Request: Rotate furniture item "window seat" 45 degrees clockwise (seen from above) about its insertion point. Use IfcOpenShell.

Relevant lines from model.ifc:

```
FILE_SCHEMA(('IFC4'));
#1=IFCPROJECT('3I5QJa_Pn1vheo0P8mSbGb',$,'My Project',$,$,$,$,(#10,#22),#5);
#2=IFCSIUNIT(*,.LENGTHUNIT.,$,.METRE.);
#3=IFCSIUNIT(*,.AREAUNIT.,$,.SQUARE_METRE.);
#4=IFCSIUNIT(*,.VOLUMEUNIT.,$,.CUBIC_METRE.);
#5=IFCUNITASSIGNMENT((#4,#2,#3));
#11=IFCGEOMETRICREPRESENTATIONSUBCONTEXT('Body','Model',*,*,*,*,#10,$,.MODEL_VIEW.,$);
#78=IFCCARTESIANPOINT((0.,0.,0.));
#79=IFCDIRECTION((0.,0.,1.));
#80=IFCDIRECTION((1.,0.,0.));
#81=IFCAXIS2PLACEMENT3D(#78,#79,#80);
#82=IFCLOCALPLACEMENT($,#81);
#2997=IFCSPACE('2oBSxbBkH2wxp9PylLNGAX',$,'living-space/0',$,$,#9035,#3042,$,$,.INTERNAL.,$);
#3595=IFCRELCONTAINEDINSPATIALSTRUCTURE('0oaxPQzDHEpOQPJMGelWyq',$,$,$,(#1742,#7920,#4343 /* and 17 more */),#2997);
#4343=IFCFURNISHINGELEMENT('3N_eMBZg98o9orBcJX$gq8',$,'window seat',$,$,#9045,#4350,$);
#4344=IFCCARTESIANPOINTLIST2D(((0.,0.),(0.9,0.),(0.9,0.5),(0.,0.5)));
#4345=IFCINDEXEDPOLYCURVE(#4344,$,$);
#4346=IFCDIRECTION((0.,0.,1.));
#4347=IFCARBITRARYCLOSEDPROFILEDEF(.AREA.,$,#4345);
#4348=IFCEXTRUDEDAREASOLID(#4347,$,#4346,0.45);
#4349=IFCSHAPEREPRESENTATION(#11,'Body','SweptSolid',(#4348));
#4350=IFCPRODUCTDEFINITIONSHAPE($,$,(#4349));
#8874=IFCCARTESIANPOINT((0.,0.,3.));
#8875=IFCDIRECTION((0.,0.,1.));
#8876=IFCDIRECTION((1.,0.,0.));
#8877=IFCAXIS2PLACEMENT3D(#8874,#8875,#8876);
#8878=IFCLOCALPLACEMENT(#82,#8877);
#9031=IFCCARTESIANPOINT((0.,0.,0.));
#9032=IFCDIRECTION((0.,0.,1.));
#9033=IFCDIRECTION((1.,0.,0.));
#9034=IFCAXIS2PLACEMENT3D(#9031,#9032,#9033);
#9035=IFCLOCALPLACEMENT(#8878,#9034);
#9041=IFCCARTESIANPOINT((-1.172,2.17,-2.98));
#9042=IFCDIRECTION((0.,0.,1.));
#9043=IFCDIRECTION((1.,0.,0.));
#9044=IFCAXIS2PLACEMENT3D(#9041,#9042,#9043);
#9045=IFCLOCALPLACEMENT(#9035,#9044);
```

```python
import ifcopenshell
import ifcopenshell.api.geometry
import ifcopenshell.util.placement

model = ifcopenshell.open("model.ifc")

item = model.by_id(4343)
matrix = ifcopenshell.util.placement.get_local_placement(item.ObjectPlacement)
matrix = matrix @ ifcopenshell.util.placement.rotation(-45, "Z")
ifcopenshell.api.geometry.edit_object_placement(model, product=item, matrix=matrix, is_si=False)

print(ifcopenshell.util.placement.get_local_placement(item.ObjectPlacement).round(3) + 0.0)

model.write("model_v2.ifc")
```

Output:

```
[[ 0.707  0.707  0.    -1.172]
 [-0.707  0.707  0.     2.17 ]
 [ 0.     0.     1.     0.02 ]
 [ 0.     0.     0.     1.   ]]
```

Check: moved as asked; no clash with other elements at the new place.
